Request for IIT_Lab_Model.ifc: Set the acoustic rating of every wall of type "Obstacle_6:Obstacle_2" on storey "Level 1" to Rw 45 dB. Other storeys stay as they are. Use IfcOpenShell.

First a look at what the model holds.

```python
import ifcopenshell
import ifcopenshell.util.element

model = ifcopenshell.open("IIT_Lab_Model.ifc")
print(model.schema)
storey = next(s for s in model.by_type("IfcBuildingStorey") if s.Name == "Level 1")
walls = [e for e in ifcopenshell.util.element.get_decomposition(storey) if e.is_a("IfcWall")]
seen = {}
for e in walls:
    element_type = ifcopenshell.util.element.get_type(e)
    key = (element_type.Name if element_type != e and element_type else None, ifcopenshell.util.element.get_pset(e, "Pset_WallCommon", "AcousticRating"))
    seen[key] = seen.get(key, 0) + 1
for (name, value), count in sorted(seen.items(), key=str):
    print(count, "x", name, "|", value)
```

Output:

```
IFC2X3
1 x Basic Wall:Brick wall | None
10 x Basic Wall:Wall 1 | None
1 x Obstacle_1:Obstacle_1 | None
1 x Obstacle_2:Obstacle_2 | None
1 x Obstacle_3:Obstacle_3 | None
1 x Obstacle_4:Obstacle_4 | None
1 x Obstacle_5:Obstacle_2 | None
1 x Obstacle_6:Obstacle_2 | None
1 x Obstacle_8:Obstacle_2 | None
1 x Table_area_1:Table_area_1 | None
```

```python
import ifcopenshell
import ifcopenshell.api.pset
import ifcopenshell.util.element

model = ifcopenshell.open("IIT_Lab_Model.ifc")

storey = next(s for s in model.by_type("IfcBuildingStorey") if s.Name == "Level 1")
walls = [e for e in ifcopenshell.util.element.get_decomposition(storey) if e.is_a("IfcWall")]

count = 0
for e in walls:
    element_type = ifcopenshell.util.element.get_type(e)
    if element_type in (None, e) or element_type.Name != "Obstacle_6:Obstacle_2":
        continue
    # add_pset returns the element's existing set when there is one.
    pset = ifcopenshell.api.pset.add_pset(model, product=e, name="Pset_WallCommon")
    ifcopenshell.api.pset.edit_pset(model, pset=pset, properties={"AcousticRating": "Rw 45 dB"})
    count += 1

print(count, "walls updated")

model.write("IIT_Lab_Model_updated.ifc")
```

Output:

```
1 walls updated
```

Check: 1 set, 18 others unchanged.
